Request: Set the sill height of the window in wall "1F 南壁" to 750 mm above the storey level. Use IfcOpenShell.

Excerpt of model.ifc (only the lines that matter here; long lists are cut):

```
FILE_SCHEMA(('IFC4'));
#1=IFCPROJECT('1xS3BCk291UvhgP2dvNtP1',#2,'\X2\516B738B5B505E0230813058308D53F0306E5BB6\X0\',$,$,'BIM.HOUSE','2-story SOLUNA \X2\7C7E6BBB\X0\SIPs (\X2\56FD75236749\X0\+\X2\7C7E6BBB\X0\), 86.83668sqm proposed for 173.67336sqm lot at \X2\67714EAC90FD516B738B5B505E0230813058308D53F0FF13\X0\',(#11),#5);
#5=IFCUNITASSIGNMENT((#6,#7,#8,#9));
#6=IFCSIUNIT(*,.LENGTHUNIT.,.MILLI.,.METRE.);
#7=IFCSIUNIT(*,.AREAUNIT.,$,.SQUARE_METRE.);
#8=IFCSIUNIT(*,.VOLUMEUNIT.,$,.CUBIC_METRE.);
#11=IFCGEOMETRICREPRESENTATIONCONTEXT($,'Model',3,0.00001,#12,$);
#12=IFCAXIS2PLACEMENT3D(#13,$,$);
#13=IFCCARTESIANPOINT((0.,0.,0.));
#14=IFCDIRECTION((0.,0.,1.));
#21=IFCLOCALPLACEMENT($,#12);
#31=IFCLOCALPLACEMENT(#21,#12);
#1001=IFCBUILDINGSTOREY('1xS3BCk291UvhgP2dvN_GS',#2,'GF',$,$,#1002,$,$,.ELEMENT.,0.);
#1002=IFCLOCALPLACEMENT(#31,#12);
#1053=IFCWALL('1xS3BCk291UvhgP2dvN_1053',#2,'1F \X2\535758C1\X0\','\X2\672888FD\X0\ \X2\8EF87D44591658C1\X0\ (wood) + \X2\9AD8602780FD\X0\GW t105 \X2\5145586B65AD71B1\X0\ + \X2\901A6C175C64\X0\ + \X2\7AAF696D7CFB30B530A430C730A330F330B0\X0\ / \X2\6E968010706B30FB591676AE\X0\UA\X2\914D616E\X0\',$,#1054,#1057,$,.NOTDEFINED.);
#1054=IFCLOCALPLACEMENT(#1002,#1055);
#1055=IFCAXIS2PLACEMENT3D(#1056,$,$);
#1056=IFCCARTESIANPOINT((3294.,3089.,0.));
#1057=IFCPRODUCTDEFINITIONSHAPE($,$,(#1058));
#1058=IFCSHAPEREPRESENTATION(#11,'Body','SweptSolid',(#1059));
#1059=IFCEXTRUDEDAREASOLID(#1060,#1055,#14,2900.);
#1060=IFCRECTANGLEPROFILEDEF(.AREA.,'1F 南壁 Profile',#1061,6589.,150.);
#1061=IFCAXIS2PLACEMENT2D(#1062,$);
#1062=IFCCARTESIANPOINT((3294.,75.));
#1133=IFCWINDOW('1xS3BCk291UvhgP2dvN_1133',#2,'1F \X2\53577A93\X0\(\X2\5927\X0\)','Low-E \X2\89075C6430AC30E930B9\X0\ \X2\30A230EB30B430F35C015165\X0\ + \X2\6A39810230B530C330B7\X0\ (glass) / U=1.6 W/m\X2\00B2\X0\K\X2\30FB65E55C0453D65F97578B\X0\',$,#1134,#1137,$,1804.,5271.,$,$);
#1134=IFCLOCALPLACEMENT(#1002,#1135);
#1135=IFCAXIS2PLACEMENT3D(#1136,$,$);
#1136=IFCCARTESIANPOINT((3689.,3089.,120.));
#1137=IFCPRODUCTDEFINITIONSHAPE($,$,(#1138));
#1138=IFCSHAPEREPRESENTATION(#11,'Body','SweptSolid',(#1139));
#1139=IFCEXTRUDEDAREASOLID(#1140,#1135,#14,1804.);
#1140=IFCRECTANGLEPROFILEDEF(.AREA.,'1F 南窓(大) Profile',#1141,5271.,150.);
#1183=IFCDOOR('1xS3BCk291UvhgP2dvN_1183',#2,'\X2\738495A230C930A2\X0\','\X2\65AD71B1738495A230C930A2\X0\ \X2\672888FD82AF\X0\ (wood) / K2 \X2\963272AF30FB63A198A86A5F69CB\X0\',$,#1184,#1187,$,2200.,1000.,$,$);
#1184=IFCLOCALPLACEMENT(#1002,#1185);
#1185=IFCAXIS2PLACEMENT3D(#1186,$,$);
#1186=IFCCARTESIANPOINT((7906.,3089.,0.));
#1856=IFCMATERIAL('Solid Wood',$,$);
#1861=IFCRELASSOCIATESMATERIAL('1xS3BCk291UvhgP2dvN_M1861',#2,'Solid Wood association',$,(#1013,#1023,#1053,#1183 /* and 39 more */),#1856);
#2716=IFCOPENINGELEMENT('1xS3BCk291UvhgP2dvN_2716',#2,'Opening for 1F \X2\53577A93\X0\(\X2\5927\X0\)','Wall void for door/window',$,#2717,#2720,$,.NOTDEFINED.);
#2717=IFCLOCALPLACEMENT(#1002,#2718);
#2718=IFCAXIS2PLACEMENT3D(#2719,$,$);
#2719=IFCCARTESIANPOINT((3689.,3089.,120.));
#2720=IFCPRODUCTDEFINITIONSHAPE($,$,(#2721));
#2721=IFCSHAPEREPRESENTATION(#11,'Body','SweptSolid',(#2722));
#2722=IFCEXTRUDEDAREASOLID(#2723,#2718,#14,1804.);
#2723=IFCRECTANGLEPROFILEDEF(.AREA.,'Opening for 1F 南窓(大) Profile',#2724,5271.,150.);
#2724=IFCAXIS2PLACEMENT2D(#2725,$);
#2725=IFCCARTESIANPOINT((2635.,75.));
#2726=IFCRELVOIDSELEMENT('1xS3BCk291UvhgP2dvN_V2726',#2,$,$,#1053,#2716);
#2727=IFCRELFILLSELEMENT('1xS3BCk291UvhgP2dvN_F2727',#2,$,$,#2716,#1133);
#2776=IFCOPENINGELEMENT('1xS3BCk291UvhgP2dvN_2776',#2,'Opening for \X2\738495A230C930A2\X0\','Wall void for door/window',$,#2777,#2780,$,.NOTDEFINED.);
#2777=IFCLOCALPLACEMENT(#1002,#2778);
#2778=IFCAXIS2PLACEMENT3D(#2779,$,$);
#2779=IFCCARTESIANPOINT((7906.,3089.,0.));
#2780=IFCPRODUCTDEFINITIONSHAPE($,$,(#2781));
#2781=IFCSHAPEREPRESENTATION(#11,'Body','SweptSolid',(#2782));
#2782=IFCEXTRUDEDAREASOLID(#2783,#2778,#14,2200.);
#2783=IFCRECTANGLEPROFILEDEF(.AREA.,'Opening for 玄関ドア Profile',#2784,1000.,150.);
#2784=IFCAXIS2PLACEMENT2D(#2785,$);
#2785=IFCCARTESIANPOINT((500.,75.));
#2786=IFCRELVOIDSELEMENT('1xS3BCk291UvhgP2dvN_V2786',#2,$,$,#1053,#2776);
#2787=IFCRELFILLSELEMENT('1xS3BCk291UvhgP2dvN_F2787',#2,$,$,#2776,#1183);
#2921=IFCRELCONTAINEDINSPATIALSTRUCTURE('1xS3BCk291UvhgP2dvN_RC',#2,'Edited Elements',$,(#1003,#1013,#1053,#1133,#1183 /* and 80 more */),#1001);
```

```python
import numpy as np
import ifcopenshell
import ifcopenshell.api.geometry
import ifcopenshell.geom
import ifcopenshell.util.element
import ifcopenshell.util.placement
import ifcopenshell.util.shape
import ifcopenshell.util.unit

model = ifcopenshell.open("model.ifc")
unit_scale = ifcopenshell.util.unit.calculate_unit_scale(model)

window = model.by_id(1133)
opening = window.FillsVoids[0].RelatingOpeningElement
storey = ifcopenshell.util.element.get_container(window, ifc_class="IfcBuildingStorey")
level = ifcopenshell.util.placement.get_local_placement(storey.ObjectPlacement)[2, 3]

# The opening's origin need not be at the sill, so measure its lowest point.
shape = ifcopenshell.geom.create_shape(ifcopenshell.geom.settings(), opening)
bottom = ifcopenshell.util.shape.get_shape_bottom_elevation(shape, shape.geometry) / unit_scale
dz = level + 0.75 / unit_scale - bottom

shift = np.array([0.0, 0.0, dz])
# The window is not placed relative to its opening, so move both.
for product in (opening, window):
    matrix = ifcopenshell.util.placement.get_local_placement(product.ObjectPlacement)
    matrix[:3, 3] += shift
    ifcopenshell.api.geometry.edit_object_placement(model, product=product, matrix=matrix, is_si=False)

print(f"moved by {dz * unit_scale:+.3f} m")

model.write("model_updated.ifc")
```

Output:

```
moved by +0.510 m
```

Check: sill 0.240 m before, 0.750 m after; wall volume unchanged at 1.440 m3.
